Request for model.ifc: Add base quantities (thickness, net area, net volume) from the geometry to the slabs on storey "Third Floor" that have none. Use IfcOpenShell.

First a look at what the model holds.

```python
import ifcopenshell
import ifcopenshell.util.element
import ifcopenshell.util.unit

model = ifcopenshell.open("model.ifc")
print(model.schema)
for unit_type in ("LENGTHUNIT", "AREAUNIT", "VOLUMEUNIT"):
    print(unit_type, ifcopenshell.util.unit.calculate_unit_scale(model, unit_type))
storey = next(s for s in model.by_type("IfcBuildingStorey") if s.Name == "Third Floor")
slabs = [e for e in ifcopenshell.util.element.get_decomposition(storey) if e.is_a("IfcSlab")]
for e in sorted(slabs, key=lambda e: e.id()):
    print(e.id(), e.is_a(), e.Name, list(ifcopenshell.util.element.get_psets(e, qtos_only=True)), sep=" | ")
```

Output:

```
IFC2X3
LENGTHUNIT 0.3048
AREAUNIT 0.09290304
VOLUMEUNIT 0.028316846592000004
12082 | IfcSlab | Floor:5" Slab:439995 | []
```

```python
import ifcopenshell
import ifcopenshell.api.pset
import ifcopenshell.geom
import ifcopenshell.util.element
import ifcopenshell.util.shape
import ifcopenshell.util.unit

model = ifcopenshell.open("model.ifc")
unit_scale = ifcopenshell.util.unit.calculate_unit_scale(model)
area_scale = ifcopenshell.util.unit.calculate_unit_scale(model, "AREAUNIT")
volume_scale = ifcopenshell.util.unit.calculate_unit_scale(model, "VOLUMEUNIT")
settings = ifcopenshell.geom.settings()

storey = next(s for s in model.by_type("IfcBuildingStorey") if s.Name == "Third Floor")
slabs = [e for e in ifcopenshell.util.element.get_decomposition(storey) if e.is_a("IfcSlab")]

for e in sorted(slabs, key=lambda e: e.id()):
    if ifcopenshell.util.element.get_psets(e, qtos_only=True, should_inherit=False):
        continue
    # Geometry comes back in metres, in the element's own axes.
    shape = ifcopenshell.geom.create_shape(settings, e)
    values = {
        "Width": ifcopenshell.util.shape.get_z(shape.geometry) / unit_scale,
        "NetArea": ifcopenshell.util.shape.get_footprint_area(shape.geometry) / area_scale,
        "NetVolume": ifcopenshell.util.shape.get_volume(shape.geometry) / volume_scale,
    }
    qto = ifcopenshell.api.pset.add_qto(model, product=e, name="BaseQuantities")
    ifcopenshell.api.pset.edit_qto(model, qto=qto, properties=values)
    print(e.id(), {k: round(v, 3) for k, v in values.items()})

model.write("model-out.ifc")
```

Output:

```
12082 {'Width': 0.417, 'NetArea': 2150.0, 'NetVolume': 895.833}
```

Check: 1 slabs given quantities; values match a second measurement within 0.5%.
